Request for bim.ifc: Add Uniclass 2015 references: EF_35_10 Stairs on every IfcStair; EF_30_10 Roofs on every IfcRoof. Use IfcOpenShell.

First a look at what the model holds.

```python
import ifcopenshell

model = ifcopenshell.open("bim.ifc")
print(model.schema)
print("classifications:", [c.Name for c in model.by_type("IfcClassification")])
for ifc_class in ("IfcDoor", "IfcRoof", "IfcStair", "IfcWall", "IfcWindow"):
    print(ifc_class, len(model.by_type(ifc_class)))
```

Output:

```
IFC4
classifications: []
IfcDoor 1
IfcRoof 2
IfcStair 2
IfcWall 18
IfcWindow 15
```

```python
import ifcopenshell
import ifcopenshell.api.classification

model = ifcopenshell.open("bim.ifc")

system = ifcopenshell.api.classification.add_classification(model, classification="Uniclass 2015")

codes = {
    "IfcStair": ("EF_35_10", "Stairs"),
    "IfcRoof": ("EF_30_10", "Roofs"),
}
for ifc_class, (code, name) in codes.items():
    products = model.by_type(ifc_class)
    ifcopenshell.api.classification.add_reference(
        model, products=products, classification=system, identification=code, name=name
    )
    print(code, len(products))

model.write("bim_updated.ifc")
```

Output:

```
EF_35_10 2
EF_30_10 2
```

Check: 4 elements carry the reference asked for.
